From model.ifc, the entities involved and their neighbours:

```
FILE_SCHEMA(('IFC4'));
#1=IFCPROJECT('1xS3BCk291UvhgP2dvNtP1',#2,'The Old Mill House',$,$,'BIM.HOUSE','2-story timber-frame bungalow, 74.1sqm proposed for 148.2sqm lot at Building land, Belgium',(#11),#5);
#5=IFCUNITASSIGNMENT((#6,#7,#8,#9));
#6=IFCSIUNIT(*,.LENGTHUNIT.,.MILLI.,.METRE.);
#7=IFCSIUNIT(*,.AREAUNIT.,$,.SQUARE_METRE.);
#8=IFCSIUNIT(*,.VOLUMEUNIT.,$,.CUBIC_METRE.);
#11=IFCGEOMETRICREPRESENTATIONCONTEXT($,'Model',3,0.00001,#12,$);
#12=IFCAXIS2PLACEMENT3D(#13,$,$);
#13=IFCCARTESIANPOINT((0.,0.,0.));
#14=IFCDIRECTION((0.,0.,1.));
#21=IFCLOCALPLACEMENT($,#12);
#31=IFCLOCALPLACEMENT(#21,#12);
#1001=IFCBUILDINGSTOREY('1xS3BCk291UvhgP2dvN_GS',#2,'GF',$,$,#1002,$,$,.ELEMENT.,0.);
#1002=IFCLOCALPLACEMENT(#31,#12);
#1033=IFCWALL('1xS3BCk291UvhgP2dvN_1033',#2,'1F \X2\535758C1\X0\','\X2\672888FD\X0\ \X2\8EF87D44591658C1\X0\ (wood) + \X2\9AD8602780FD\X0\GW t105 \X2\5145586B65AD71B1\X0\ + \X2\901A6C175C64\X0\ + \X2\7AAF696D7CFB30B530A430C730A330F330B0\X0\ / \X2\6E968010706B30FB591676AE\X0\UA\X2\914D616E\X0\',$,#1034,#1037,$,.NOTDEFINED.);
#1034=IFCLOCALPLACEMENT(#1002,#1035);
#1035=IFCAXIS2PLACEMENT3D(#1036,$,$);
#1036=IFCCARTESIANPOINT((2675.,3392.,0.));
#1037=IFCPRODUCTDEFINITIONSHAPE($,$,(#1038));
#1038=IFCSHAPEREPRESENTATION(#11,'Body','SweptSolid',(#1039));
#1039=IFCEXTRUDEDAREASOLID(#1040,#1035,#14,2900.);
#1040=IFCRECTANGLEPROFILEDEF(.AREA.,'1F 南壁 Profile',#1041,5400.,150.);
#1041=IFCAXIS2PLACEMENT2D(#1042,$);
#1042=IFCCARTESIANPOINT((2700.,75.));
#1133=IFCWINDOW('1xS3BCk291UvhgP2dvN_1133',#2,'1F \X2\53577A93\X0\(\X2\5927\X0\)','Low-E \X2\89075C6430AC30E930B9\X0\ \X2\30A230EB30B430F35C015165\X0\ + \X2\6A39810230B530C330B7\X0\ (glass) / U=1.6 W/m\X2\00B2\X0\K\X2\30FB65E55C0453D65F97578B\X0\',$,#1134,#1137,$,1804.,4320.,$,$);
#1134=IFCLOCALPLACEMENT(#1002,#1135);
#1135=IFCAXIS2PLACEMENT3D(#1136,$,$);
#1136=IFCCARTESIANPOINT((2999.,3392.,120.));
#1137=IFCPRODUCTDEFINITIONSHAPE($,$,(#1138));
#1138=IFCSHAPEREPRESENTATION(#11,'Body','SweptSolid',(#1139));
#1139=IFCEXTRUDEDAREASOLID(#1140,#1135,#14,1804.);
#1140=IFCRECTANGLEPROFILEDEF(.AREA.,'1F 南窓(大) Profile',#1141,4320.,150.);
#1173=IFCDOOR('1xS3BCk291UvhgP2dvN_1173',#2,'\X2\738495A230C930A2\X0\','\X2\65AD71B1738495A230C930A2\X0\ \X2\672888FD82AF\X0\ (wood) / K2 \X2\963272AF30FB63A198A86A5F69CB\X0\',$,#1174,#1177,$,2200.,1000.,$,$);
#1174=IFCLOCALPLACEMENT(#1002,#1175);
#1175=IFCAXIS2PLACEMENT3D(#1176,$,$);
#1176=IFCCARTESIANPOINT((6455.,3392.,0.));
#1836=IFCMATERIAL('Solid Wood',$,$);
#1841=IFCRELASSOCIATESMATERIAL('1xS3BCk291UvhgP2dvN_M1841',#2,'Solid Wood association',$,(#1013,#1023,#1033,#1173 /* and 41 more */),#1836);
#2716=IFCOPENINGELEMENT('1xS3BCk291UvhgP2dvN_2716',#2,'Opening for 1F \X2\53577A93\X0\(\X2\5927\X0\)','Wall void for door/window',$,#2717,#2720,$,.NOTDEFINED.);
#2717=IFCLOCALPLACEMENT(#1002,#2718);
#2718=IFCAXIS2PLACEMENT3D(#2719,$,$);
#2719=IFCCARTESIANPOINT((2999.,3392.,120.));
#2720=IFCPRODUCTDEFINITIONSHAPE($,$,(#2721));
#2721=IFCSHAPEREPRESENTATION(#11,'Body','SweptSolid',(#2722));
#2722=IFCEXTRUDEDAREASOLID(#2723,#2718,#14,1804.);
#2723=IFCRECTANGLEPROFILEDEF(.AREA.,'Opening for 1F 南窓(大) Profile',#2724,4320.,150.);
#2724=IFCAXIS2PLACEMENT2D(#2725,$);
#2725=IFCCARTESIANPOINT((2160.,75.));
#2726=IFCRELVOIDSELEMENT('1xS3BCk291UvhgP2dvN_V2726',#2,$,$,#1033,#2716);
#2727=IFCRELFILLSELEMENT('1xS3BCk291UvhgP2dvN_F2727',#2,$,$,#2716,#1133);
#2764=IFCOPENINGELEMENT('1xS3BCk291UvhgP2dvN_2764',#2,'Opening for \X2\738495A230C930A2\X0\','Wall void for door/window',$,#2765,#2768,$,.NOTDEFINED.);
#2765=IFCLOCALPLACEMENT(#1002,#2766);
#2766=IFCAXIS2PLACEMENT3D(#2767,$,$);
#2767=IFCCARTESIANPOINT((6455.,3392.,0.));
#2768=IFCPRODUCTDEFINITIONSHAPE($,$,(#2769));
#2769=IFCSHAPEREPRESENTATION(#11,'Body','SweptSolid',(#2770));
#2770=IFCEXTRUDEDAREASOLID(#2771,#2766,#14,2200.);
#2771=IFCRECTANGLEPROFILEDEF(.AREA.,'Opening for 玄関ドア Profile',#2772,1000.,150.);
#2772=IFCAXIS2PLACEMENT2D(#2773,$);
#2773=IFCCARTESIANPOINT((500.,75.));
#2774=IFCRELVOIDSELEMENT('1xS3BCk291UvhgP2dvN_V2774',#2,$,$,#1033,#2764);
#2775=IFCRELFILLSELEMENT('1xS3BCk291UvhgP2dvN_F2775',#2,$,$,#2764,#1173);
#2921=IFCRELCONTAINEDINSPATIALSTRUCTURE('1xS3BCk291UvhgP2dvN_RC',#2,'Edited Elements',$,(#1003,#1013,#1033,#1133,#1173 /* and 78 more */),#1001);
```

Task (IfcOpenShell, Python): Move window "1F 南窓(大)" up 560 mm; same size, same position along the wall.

```python
import numpy as np
import ifcopenshell
import ifcopenshell.api.geometry
import ifcopenshell.util.placement
import ifcopenshell.util.unit

model = ifcopenshell.open("model.ifc")
unit_scale = ifcopenshell.util.unit.calculate_unit_scale(model)

window = model.by_id(1133)
opening = window.FillsVoids[0].RelatingOpeningElement
dz = 0.56 / unit_scale

shift = np.array([0.0, 0.0, dz])
# The window is not placed relative to its opening, so move both.
for product in (opening, window):
    matrix = ifcopenshell.util.placement.get_local_placement(product.ObjectPlacement)
    matrix[:3, 3] += shift
    ifcopenshell.api.geometry.edit_object_placement(model, product=product, matrix=matrix, is_si=False)

print(f"moved by {dz * unit_scale:+.3f} m")

model.write("model-out.ifc")
```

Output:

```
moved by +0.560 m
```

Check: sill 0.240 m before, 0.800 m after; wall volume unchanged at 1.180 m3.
